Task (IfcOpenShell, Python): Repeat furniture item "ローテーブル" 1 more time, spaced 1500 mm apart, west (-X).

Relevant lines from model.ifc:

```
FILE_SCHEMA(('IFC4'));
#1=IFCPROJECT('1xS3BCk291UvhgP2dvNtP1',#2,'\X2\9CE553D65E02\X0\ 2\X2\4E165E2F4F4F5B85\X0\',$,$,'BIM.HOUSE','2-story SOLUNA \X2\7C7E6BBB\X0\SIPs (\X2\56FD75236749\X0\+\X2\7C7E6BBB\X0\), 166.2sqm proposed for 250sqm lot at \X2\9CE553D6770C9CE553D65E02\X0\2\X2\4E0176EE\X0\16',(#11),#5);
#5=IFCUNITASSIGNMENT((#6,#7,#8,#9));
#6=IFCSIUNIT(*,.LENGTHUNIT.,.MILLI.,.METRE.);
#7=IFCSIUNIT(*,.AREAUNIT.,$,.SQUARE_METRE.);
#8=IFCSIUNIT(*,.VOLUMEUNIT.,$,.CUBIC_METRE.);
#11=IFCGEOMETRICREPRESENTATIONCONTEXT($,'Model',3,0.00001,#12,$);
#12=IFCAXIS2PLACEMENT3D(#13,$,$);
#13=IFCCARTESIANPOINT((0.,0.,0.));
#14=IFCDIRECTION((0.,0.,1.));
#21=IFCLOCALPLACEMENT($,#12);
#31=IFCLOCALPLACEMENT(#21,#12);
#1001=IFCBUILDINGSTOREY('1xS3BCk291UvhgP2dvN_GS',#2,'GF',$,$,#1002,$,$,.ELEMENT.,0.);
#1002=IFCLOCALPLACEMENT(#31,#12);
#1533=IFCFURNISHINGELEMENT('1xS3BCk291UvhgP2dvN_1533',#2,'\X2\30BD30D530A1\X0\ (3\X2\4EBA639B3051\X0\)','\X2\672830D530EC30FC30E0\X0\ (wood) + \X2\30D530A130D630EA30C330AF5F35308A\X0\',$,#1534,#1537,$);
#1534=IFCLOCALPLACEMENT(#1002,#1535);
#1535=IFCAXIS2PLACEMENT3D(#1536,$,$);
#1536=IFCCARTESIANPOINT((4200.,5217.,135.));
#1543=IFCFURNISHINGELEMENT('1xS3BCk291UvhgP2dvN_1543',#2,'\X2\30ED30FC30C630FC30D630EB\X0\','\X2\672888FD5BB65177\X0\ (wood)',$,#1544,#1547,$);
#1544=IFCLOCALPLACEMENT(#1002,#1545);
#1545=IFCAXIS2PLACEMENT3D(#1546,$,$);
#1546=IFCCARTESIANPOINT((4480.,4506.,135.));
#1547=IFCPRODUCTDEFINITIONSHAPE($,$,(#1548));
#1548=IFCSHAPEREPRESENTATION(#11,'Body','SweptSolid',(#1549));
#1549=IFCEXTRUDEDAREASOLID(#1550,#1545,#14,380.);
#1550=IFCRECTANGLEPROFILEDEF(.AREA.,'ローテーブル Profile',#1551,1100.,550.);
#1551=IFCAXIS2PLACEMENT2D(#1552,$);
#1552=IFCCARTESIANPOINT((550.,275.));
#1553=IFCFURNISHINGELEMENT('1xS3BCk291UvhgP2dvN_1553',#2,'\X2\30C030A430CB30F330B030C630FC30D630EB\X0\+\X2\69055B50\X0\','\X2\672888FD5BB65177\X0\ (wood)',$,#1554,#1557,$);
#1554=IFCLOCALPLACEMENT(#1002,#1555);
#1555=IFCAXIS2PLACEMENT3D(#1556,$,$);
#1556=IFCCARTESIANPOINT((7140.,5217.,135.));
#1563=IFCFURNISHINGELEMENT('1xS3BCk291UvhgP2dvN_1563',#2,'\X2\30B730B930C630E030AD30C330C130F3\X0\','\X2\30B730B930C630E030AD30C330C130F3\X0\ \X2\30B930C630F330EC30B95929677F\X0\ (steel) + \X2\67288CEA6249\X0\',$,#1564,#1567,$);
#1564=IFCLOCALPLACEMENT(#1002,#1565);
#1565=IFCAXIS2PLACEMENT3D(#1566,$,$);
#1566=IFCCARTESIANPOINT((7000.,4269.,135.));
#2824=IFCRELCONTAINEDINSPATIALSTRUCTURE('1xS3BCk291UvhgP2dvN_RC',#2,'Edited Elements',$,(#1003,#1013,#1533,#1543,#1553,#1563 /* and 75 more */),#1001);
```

```python
import numpy as np
import ifcopenshell
import ifcopenshell.api.geometry
import ifcopenshell.api.root
import ifcopenshell.util.element
import ifcopenshell.util.placement
import ifcopenshell.util.unit

model = ifcopenshell.open("model.ifc")
unit_scale = ifcopenshell.util.unit.calculate_unit_scale(model)


def reuse_history(source, copy):
    """copy_class also copies each property set's owner history, people and application; keep the originals."""
    for rel in copy.IsDefinedBy:
        if rel.is_a("IfcRelDefinesByProperties") and (history := rel.RelatingPropertyDefinition.OwnerHistory):
            rel.RelatingPropertyDefinition.OwnerHistory = source.OwnerHistory
            ifcopenshell.util.element.remove_deep2(model, history)


source = model.by_id(1543)
base = ifcopenshell.util.placement.get_local_placement(source.ObjectPlacement)
step = np.array([-1.0, 0.0, 0.0]) * 1.5 / unit_scale

for i in range(1, 2):
    copy = ifcopenshell.api.root.copy_class(model, product=source)
    copy.Representation = ifcopenshell.util.element.copy_deep(
        model, source.Representation, exclude=["IfcGeometricRepresentationContext", "IfcRepresentationMap"]
    )
    reuse_history(source, copy)
    matrix = base.copy()
    matrix[:3, 3] += i * step
    print("added at", matrix[:3, 3].round(3) + 0.0)
    ifcopenshell.api.geometry.edit_object_placement(model, product=copy, matrix=matrix, is_si=False)

model.write("model_updated.ifc")
```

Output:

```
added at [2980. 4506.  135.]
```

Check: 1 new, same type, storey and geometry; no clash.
